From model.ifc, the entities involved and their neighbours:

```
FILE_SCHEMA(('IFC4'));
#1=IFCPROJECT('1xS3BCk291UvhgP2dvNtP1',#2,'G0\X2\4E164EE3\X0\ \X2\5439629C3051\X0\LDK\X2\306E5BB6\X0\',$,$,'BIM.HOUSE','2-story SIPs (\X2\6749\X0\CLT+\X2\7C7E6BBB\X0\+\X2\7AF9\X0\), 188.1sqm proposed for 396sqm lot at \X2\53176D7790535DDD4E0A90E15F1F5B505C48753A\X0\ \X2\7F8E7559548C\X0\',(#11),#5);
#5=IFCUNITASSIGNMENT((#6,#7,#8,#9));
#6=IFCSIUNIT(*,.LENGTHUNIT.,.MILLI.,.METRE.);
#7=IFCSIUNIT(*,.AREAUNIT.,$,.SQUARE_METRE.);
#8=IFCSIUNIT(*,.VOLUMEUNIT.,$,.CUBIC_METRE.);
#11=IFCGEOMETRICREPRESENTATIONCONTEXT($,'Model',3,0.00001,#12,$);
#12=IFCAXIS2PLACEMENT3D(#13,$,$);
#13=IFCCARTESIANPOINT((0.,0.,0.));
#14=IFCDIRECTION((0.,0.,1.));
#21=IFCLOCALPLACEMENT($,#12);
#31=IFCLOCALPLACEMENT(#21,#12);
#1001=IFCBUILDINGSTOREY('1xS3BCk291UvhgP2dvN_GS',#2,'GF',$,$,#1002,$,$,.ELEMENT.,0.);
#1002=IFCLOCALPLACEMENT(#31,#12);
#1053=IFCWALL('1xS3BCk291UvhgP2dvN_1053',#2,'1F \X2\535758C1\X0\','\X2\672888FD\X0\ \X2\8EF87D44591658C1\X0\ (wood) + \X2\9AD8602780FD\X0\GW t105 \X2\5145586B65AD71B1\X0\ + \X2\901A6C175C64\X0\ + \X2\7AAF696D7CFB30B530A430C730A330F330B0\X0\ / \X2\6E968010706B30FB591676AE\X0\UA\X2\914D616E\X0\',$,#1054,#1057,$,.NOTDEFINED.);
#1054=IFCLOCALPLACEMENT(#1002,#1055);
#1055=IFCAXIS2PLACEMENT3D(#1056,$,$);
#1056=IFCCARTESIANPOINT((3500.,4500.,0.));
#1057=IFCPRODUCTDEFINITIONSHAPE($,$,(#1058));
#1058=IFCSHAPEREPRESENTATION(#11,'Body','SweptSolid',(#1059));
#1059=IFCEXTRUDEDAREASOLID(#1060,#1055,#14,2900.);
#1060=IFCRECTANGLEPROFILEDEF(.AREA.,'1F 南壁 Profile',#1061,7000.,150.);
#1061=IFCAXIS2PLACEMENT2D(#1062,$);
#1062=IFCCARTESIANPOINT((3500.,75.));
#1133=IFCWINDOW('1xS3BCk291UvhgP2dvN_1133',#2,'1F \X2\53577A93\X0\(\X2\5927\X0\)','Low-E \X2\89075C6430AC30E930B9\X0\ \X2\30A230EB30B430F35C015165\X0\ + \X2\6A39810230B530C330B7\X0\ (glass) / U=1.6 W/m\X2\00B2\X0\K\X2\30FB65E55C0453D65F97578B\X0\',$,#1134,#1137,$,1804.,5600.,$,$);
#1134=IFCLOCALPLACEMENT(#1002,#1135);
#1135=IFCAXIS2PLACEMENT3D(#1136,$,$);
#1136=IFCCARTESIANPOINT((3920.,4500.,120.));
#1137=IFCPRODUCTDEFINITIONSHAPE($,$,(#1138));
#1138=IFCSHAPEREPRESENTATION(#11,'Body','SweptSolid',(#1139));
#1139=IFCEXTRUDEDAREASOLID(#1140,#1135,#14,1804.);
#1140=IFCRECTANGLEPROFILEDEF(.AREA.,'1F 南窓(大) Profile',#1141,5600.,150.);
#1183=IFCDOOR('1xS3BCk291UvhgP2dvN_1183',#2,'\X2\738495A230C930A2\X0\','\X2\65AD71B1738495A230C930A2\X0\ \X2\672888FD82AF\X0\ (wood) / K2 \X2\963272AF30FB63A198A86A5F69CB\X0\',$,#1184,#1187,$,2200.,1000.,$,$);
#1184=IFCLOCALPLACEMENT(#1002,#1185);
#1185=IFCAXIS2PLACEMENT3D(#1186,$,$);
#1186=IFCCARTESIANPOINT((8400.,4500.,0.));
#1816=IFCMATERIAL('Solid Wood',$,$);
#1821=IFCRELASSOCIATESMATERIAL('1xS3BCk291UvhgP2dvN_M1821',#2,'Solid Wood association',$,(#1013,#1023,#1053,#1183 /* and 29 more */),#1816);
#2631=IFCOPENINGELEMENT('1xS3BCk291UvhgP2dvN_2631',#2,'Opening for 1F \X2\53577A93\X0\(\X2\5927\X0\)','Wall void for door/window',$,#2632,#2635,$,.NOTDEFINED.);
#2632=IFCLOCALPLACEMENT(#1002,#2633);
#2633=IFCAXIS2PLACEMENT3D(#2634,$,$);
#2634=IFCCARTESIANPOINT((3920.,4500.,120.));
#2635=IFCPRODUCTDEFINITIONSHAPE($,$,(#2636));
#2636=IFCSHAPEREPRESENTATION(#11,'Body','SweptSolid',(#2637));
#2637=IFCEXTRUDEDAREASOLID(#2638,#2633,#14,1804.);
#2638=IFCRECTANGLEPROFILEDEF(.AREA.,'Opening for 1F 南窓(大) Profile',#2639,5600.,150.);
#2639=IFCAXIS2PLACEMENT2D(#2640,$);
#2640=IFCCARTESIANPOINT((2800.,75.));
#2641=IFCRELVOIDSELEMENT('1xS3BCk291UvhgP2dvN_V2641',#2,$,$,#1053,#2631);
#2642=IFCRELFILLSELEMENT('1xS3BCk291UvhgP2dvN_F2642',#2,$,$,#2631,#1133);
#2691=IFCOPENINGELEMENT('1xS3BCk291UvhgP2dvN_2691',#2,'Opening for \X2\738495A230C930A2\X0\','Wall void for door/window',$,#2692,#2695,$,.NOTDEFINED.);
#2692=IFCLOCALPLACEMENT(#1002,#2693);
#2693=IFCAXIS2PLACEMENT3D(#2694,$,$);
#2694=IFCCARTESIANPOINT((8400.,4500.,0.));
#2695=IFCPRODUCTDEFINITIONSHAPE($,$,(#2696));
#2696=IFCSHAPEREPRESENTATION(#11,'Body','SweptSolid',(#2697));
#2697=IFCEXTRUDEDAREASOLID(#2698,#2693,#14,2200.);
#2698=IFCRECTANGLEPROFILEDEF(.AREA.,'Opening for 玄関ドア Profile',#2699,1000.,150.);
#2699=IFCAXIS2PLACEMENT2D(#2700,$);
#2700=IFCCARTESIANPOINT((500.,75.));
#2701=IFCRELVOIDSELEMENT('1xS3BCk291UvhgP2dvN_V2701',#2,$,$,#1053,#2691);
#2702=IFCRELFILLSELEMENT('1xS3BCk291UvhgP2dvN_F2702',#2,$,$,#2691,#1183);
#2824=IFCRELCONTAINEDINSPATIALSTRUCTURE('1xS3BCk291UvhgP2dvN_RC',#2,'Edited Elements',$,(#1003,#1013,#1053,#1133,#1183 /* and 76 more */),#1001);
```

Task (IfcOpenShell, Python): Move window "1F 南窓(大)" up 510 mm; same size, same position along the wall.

```python
import numpy as np
import ifcopenshell
import ifcopenshell.api.geometry
import ifcopenshell.util.placement
import ifcopenshell.util.unit

model = ifcopenshell.open("model.ifc")
unit_scale = ifcopenshell.util.unit.calculate_unit_scale(model)

window = model.by_guid("1xS3BCk291UvhgP2dvN_1133")
opening = window.FillsVoids[0].RelatingOpeningElement
dz = 510.0

shift = np.array([0.0, 0.0, dz])
# The window is not placed relative to its opening, so move both.
for product in (opening, window):
    matrix = ifcopenshell.util.placement.get_local_placement(product.ObjectPlacement)
    matrix[:3, 3] += shift
    ifcopenshell.api.geometry.edit_object_placement(model, product=product, matrix=matrix, is_si=False)

print(f"moved by {dz * unit_scale:+.3f} m")

model.write("model-out.ifc")
```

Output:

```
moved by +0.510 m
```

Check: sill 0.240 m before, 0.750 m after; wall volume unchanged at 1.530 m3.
